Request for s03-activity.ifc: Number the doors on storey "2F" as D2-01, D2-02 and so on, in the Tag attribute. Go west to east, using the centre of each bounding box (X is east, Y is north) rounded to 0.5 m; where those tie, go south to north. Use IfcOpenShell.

First a look at what the model holds.

```python
import ifcopenshell
import ifcopenshell.util.element
import ifcopenshell.util.placement

model = ifcopenshell.open("s03-activity.ifc")
print(model.schema)
storey = next(s for s in model.by_type("IfcBuildingStorey") if s.Name == "2F")
doors = [e for e in ifcopenshell.util.element.get_decomposition(storey) if e.is_a("IfcDoor")]
for e in sorted(doors, key=lambda e: e.id()):
    origin = ifcopenshell.util.placement.get_local_placement(e.ObjectPlacement)[:3, 3]
    print(e.id(), e.Tag, e.Name, origin.round(2) + 0.0, sep=" | ")
```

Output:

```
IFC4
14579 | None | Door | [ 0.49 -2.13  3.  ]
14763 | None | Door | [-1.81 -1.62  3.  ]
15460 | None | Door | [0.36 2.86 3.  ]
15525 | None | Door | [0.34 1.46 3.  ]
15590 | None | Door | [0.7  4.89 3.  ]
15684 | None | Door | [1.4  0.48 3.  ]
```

```python
import ifcopenshell
import ifcopenshell.geom
import ifcopenshell.util.element
import ifcopenshell.util.shape

model = ifcopenshell.open("s03-activity.ifc")
settings = ifcopenshell.geom.settings()
settings.set("use-world-coords", True)


def centre(element):
    shape = ifcopenshell.geom.create_shape(settings, element)
    return ifcopenshell.util.shape.get_bbox_centroid(shape.geometry)


storey = next(s for s in model.by_type("IfcBuildingStorey") if s.Name == "2F")
doors = [e for e in ifcopenshell.util.element.get_decomposition(storey) if e.is_a("IfcDoor")]

# Insertion points can sit at a corner or the storey origin, so sort by the geometry (in metres).
centres = {e: centre(e) for e in doors}
doors.sort(key=lambda e: (round(centres[e][0] / 0.5), centres[e][1]))

for i, e in enumerate(doors, start=1):
    number = f"D2-{i:02d}"
    e.Tag = number
    print(e.id(), number)

model.write("s03-activity_rev.ifc")
```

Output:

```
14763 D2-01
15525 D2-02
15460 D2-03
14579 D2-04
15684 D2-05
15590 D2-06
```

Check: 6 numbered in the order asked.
